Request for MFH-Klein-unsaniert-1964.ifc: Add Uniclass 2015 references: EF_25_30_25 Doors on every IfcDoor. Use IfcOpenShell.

First a look at what the model holds.

```python
import ifcopenshell

model = ifcopenshell.open("MFH-Klein-unsaniert-1964.ifc")
print(model.schema)
print("classifications:", [c.Name for c in model.by_type("IfcClassification")])
for ifc_class in ("IfcDoor", "IfcRoof", "IfcStair", "IfcWall", "IfcWindow"):
    print(ifc_class, len(model.by_type(ifc_class)))
```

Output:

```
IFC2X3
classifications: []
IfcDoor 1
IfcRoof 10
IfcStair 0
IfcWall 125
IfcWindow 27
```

```python
import ifcopenshell
import ifcopenshell.api.classification

model = ifcopenshell.open("MFH-Klein-unsaniert-1964.ifc")

# IFC2X3 requires Source and Edition and has no link from the project to the system.
system = model.create_entity("IfcClassification", Source="NBS", Edition="2015", Name="Uniclass 2015")

codes = {
    "IfcDoor": ("EF_25_30_25", "Doors"),
}
for ifc_class, (code, name) in codes.items():
    products = model.by_type(ifc_class)
    ifcopenshell.api.classification.add_reference(
        model, products=products, classification=system, identification=code, name=name
    )
    print(code, len(products))

model.write("MFH-Klein-unsaniert-1964_rev.ifc")
```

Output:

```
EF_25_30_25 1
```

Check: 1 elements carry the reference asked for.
